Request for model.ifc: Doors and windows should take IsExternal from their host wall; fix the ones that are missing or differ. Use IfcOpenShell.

First a look at what the model holds.

```python
import ifcopenshell
import ifcopenshell.util.element

model = ifcopenshell.open("model.ifc")
print(model.schema)
seen = {}
for e in model.by_type("IfcDoor") + model.by_type("IfcWindow"):
    if not e.FillsVoids:
        continue
    host = e.FillsVoids[0].RelatingOpeningElement.VoidsElements[0].RelatingBuildingElement
    own = ifcopenshell.util.element.get_pset(e, f"Pset_{e.is_a()[3:].removesuffix('StandardCase')}Common", "IsExternal")
    wall = ifcopenshell.util.element.get_pset(host, "Pset_WallCommon", "IsExternal")
    seen[e.is_a(), own, wall] = seen.get((e.is_a(), own, wall), 0) + 1
for (cls, own, wall), count in sorted(seen.items(), key=str):
    print(count, cls, "IsExternal:", own, "| host wall:", wall)
```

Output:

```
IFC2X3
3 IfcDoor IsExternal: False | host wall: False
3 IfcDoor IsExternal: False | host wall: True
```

```python
import ifcopenshell
import ifcopenshell.api.pset
import ifcopenshell.util.element

model = ifcopenshell.open("model.ifc")

count = 0
for ifc_class, pset_name in (("IfcDoor", "Pset_DoorCommon"), ("IfcWindow", "Pset_WindowCommon")):
    for e in model.by_type(ifc_class):
        if not e.FillsVoids:
            continue
        host = e.FillsVoids[0].RelatingOpeningElement.VoidsElements[0].RelatingBuildingElement
        external = ifcopenshell.util.element.get_pset(host, "Pset_WallCommon", "IsExternal")
        if external is None or ifcopenshell.util.element.get_pset(e, pset_name, "IsExternal") == external:
            continue
        pset = ifcopenshell.api.pset.add_pset(model, product=e, name=pset_name)
        ifcopenshell.api.pset.edit_pset(model, pset=pset, properties={"IsExternal": external})
        count += 1

print(count, "updated")

model.write("model_v2.ifc")
```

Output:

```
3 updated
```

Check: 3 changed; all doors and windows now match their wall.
